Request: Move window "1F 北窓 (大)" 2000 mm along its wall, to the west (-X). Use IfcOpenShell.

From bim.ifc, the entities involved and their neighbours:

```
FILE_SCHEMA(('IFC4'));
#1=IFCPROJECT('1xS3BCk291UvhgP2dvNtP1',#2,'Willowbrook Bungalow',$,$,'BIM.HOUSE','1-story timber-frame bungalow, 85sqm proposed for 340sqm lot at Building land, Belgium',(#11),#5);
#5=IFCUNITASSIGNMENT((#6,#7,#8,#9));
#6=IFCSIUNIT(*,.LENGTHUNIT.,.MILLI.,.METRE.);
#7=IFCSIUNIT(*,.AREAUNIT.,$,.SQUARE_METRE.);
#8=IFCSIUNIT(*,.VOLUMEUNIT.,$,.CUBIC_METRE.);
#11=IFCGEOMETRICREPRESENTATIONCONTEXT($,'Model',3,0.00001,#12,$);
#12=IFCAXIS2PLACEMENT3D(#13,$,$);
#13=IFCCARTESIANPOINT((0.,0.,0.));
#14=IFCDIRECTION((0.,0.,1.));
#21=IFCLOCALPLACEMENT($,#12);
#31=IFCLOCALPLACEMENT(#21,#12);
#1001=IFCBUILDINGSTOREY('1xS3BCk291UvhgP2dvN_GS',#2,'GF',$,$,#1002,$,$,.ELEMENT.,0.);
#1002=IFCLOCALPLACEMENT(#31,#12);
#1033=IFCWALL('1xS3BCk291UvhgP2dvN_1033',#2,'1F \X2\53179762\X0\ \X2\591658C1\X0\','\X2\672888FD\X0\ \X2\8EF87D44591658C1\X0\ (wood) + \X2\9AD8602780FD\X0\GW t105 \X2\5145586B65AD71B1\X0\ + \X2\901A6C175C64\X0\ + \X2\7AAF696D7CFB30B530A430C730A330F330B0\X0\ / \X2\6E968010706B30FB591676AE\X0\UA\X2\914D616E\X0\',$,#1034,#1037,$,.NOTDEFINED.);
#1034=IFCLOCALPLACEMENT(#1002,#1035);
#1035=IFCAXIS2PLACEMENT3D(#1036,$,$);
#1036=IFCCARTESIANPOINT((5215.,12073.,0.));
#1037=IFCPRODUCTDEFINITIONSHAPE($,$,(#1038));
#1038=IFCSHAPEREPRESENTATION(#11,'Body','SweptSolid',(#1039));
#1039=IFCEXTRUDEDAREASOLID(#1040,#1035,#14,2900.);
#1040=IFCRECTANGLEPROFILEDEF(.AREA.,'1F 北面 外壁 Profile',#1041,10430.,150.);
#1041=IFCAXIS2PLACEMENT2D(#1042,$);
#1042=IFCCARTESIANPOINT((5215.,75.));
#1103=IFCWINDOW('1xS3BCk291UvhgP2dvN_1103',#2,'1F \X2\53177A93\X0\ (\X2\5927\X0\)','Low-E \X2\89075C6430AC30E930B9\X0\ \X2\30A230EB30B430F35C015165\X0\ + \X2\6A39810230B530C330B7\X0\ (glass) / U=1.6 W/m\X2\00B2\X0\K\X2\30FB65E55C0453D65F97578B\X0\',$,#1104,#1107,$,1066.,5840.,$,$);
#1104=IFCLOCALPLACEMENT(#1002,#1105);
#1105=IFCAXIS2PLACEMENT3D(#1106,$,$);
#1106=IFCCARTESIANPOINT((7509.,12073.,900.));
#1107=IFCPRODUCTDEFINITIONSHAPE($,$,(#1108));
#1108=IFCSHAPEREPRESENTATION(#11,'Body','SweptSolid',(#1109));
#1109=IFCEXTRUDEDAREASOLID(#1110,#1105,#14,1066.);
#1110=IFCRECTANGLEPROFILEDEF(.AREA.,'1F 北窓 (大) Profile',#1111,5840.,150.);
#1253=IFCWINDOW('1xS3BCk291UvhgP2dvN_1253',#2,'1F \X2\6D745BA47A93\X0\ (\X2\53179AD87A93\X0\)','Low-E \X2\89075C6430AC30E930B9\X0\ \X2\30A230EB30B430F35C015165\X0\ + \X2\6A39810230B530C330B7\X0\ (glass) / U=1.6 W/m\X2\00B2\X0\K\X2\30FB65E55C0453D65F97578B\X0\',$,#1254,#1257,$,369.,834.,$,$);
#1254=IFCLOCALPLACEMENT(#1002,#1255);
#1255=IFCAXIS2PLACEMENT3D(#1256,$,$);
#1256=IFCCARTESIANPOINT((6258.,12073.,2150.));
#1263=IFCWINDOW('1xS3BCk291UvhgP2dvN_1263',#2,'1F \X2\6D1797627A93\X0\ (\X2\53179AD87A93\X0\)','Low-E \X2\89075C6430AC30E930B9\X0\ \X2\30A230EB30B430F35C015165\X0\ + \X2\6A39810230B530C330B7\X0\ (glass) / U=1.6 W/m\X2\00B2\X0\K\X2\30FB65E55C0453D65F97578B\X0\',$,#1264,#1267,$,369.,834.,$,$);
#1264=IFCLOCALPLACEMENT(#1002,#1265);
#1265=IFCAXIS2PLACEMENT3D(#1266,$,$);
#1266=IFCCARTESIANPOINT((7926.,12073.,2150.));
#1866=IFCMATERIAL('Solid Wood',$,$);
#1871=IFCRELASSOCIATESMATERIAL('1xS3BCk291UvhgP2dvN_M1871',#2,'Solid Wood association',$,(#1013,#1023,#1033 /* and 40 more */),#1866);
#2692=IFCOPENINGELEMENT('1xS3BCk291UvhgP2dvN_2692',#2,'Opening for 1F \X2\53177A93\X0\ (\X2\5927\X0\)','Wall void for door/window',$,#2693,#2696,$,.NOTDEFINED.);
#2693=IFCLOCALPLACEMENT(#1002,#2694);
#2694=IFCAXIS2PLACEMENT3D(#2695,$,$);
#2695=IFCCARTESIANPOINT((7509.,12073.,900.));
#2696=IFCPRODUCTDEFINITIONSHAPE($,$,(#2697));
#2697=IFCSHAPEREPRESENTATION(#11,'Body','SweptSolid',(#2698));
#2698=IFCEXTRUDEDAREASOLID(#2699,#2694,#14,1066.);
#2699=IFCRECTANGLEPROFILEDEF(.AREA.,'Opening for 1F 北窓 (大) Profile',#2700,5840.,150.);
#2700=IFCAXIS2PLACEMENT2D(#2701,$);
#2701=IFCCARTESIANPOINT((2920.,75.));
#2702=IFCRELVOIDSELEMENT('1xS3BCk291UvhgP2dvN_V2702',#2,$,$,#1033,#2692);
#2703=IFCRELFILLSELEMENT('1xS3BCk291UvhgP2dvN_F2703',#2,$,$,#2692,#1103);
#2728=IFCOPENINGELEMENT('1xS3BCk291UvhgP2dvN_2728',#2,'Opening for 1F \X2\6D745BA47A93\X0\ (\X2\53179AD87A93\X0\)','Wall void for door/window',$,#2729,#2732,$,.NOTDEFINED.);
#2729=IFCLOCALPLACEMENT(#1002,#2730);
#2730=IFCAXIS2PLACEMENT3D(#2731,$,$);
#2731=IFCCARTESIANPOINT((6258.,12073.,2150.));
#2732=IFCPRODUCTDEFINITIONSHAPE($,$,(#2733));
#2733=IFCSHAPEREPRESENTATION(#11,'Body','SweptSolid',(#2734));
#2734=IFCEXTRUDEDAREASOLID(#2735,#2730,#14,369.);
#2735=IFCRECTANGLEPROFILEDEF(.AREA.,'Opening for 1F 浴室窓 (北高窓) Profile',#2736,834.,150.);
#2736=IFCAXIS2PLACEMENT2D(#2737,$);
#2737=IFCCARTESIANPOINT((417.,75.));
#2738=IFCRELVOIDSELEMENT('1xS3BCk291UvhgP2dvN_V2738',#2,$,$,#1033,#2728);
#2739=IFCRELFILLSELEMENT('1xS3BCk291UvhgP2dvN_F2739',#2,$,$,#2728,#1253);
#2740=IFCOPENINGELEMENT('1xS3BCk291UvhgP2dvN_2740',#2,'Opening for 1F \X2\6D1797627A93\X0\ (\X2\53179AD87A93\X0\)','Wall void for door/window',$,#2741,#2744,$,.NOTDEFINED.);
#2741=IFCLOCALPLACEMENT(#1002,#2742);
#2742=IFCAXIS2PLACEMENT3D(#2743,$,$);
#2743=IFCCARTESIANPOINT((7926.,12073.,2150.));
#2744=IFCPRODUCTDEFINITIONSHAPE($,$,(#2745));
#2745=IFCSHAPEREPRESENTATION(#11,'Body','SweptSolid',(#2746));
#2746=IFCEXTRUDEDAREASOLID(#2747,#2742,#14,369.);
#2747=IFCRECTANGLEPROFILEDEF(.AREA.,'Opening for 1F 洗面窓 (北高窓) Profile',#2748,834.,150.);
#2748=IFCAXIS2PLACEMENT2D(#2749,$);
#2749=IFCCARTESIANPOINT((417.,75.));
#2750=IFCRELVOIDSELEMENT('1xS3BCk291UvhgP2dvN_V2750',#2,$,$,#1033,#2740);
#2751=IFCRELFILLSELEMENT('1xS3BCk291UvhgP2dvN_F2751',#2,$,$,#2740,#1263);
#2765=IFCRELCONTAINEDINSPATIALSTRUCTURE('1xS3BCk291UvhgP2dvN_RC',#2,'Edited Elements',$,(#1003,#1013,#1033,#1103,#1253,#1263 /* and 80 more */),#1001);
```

```python
import ifcopenshell
import ifcopenshell.api.geometry
import ifcopenshell.util.placement
import ifcopenshell.util.unit

model = ifcopenshell.open("bim.ifc")
unit_scale = ifcopenshell.util.unit.calculate_unit_scale(model)

window = model.by_guid("1xS3BCk291UvhgP2dvN_1103")
opening = window.FillsVoids[0].RelatingOpeningElement
wall = opening.VoidsElements[0].RelatingBuildingElement

wall_matrix = ifcopenshell.util.placement.get_local_placement(wall.ObjectPlacement)
shift = wall_matrix[:3, 0] * -2 / unit_scale
before = ifcopenshell.util.placement.get_local_placement(window.ObjectPlacement)[:3, 3].copy()

# The window is not placed relative to its opening, so move both.
for product in (opening, window):
    matrix = ifcopenshell.util.placement.get_local_placement(product.ObjectPlacement)
    matrix[:3, 3] += shift
    ifcopenshell.api.geometry.edit_object_placement(model, product=product, matrix=matrix, is_si=False)

after = ifcopenshell.util.placement.get_local_placement(window.ObjectPlacement)[:3, 3]
print("window moved by", (after - before).round(3) + 0.0)

model.write("bim_updated.ifc")
```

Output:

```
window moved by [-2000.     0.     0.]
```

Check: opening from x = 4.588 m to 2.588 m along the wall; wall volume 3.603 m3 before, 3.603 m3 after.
